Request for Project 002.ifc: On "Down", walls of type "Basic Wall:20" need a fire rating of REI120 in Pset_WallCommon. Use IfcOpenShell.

First a look at what the model holds.

```python
import ifcopenshell
import ifcopenshell.util.element

model = ifcopenshell.open("Project 002.ifc")
print(model.schema)
storey = next(s for s in model.by_type("IfcBuildingStorey") if s.Name == "Down")
walls = [e for e in ifcopenshell.util.element.get_decomposition(storey) if e.is_a("IfcWall")]
seen = {}
for e in walls:
    element_type = ifcopenshell.util.element.get_type(e)
    key = (element_type.Name if element_type != e and element_type else None, ifcopenshell.util.element.get_pset(e, "Pset_WallCommon", "FireRating"))
    seen[key] = seen.get(key, 0) + 1
for (name, value), count in sorted(seen.items(), key=str):
    print(count, "x", name, "|", value)
```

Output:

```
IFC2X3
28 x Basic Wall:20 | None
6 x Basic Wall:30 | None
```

```python
import ifcopenshell
import ifcopenshell.api.pset
import ifcopenshell.util.element

model = ifcopenshell.open("Project 002.ifc")

storey = next(s for s in model.by_type("IfcBuildingStorey") if s.Name == "Down")
walls = [e for e in ifcopenshell.util.element.get_decomposition(storey) if e.is_a("IfcWall")]

count = 0
for e in walls:
    element_type = ifcopenshell.util.element.get_type(e)
    if element_type in (None, e) or element_type.Name != "Basic Wall:20":
        continue
    # add_pset returns the element's existing set when there is one.
    pset = ifcopenshell.api.pset.add_pset(model, product=e, name="Pset_WallCommon")
    ifcopenshell.api.pset.edit_pset(model, pset=pset, properties={"FireRating": "REI120"})
    count += 1

print(count, "walls updated")

model.write("Project 002-out.ifc")
```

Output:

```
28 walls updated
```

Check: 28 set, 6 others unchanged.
